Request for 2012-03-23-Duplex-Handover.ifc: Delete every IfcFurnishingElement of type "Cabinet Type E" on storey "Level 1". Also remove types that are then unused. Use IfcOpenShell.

First a look at what the model holds.

```python
import ifcopenshell
import ifcopenshell.util.element

model = ifcopenshell.open("2012-03-23-Duplex-Handover.ifc")
print(model.schema)
storey = next(s for s in model.by_type("IfcBuildingStorey") if s.Name == "Level 1")
furniture = [e for e in ifcopenshell.util.element.get_decomposition(storey) if e.is_a("IfcFurnishingElement")]
seen = {}
for e in furniture:
    element_type = ifcopenshell.util.element.get_type(e)
    name = element_type.Name if element_type not in (None, e) else None
    seen[name] = seen.get(name, 0) + 1
for name, count in sorted(seen.items(), key=str):
    print(count, "x", name)
```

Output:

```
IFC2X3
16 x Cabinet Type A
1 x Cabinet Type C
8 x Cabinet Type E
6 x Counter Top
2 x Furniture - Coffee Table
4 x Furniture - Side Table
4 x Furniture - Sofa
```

```python
import ifcopenshell
import ifcopenshell.api.root
import ifcopenshell.util.element

model = ifcopenshell.open("2012-03-23-Duplex-Handover.ifc")

storey = next(s for s in model.by_type("IfcBuildingStorey") if s.Name == "Level 1")
furniture = [e for e in ifcopenshell.util.element.get_decomposition(storey) if e.is_a("IfcFurnishingElement")]
targets = [e for e in furniture if (t := ifcopenshell.util.element.get_type(e)) not in (None, e) and t.Name == "Cabinet Type E"]
types = {ifcopenshell.util.element.get_type(e) for e in targets} - {None, *targets}

for e in targets:
    ifcopenshell.api.root.remove_product(model, product=e)
print(len(targets), "removed")

unused = [t for t in types if not ifcopenshell.util.element.get_types(t)]
for t in unused:
    ifcopenshell.api.root.remove_product(model, product=t)
print(len(unused), "unused types removed")

model.write("2012-03-23-Duplex-Handover_v2.ifc")
```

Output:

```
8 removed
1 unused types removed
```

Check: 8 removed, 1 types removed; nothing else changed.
